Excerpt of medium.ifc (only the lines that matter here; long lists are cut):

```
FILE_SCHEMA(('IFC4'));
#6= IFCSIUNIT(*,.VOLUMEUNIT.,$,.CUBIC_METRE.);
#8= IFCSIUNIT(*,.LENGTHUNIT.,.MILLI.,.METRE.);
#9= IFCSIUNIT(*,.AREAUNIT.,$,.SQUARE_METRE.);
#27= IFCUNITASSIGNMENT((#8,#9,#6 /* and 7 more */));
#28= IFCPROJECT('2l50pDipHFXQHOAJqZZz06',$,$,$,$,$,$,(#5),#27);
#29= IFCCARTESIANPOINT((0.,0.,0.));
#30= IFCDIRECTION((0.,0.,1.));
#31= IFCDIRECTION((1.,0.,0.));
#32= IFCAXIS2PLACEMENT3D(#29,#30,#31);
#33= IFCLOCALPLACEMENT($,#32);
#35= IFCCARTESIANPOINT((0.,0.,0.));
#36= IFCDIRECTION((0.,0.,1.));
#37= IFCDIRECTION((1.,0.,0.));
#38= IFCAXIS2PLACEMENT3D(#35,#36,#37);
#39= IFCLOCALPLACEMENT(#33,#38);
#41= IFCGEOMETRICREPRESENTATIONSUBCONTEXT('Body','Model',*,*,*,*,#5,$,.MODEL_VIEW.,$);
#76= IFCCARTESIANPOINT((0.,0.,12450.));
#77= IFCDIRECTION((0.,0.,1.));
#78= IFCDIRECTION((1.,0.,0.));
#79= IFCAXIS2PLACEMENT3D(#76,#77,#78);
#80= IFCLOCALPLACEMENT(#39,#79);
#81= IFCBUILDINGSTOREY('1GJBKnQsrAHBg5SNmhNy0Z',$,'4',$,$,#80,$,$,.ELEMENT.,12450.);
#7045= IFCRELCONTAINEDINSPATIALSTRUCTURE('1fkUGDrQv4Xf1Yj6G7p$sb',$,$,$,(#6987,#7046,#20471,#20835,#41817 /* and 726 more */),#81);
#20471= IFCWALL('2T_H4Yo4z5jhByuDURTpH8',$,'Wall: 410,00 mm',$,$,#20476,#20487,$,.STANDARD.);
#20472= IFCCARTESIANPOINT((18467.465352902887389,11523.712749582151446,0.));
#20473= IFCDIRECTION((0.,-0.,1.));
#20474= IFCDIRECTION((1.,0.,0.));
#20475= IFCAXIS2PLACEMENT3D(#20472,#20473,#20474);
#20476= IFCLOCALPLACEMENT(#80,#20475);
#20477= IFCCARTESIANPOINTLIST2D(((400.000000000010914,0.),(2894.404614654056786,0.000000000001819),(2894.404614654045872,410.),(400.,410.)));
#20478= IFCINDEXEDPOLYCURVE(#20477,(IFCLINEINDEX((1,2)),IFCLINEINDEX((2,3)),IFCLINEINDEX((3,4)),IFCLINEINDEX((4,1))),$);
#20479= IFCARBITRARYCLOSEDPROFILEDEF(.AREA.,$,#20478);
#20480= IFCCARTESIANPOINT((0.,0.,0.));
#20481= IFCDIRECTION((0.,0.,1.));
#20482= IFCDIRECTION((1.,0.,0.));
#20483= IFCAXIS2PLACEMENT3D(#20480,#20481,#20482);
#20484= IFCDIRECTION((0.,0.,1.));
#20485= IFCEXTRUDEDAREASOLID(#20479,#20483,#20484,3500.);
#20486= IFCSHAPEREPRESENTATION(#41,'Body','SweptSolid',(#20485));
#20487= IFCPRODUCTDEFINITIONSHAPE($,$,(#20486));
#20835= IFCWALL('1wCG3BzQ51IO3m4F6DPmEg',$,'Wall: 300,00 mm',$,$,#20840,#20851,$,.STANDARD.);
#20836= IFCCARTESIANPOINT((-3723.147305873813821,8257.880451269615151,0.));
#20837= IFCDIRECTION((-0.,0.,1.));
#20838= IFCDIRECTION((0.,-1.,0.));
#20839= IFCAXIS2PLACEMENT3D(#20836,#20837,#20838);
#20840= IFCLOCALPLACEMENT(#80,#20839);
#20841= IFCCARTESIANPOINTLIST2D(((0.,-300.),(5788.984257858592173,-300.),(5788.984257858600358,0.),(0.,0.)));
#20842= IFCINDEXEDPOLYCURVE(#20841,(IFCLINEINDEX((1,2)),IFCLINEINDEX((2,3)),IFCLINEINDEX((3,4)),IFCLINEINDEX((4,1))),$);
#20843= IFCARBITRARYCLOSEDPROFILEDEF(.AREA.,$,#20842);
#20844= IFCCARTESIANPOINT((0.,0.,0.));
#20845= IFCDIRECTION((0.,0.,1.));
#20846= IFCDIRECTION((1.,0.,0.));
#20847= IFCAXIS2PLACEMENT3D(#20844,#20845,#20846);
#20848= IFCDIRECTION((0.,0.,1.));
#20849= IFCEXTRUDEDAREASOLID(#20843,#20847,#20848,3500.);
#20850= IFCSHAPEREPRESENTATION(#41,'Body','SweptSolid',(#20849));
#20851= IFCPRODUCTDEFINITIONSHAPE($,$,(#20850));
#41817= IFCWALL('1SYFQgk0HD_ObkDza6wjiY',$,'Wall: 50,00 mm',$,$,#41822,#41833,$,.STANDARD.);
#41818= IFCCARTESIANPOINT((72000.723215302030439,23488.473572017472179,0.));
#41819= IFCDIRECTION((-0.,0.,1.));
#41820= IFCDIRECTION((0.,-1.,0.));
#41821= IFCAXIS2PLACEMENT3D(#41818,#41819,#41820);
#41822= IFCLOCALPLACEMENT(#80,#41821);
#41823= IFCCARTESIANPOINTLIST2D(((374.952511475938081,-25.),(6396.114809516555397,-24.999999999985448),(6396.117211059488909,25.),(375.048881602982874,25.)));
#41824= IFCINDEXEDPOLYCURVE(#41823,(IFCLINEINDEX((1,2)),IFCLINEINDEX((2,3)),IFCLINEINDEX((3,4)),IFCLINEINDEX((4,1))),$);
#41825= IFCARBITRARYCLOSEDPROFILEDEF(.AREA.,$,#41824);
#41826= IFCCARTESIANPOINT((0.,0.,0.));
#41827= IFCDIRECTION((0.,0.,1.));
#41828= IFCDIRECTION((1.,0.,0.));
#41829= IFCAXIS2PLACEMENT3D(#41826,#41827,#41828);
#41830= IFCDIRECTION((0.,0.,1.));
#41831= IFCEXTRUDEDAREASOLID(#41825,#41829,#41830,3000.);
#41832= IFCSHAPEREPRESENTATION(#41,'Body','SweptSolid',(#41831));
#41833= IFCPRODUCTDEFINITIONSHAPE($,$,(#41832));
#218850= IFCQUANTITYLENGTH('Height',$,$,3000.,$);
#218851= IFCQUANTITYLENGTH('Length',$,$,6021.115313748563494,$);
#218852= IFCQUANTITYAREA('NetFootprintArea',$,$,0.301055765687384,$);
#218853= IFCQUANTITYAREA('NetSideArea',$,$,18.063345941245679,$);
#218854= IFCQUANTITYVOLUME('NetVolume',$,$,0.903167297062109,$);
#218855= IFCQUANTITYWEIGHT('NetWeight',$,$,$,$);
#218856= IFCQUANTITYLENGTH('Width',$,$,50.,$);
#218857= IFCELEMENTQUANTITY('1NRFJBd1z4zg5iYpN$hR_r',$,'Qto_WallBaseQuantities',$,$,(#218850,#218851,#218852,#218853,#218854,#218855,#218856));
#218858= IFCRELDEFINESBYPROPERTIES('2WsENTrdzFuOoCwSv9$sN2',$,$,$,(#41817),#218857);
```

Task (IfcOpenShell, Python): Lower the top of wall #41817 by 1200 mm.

```python
import ifcopenshell
import ifcopenshell.api.pset
import ifcopenshell.geom
import ifcopenshell.util.element
import ifcopenshell.util.representation
import ifcopenshell.util.shape
import ifcopenshell.util.unit

model = ifcopenshell.open("medium.ifc")
area_scale = ifcopenshell.util.unit.calculate_unit_scale(model, "AREAUNIT")
volume_scale = ifcopenshell.util.unit.calculate_unit_scale(model, "VOLUMEUNIT")
settings = ifcopenshell.geom.settings()


def volume(element):
    """Net volume in cubic metres, openings subtracted."""
    shape = ifcopenshell.geom.create_shape(settings, element)
    return ifcopenshell.util.shape.get_volume(shape.geometry)


wall = model.by_guid("1SYFQgk0HD_ObkDza6wjiY")
before = volume(wall)

body = ifcopenshell.util.representation.get_representation(wall, "Model", "Body")
solid = body.Items[0]
old_height = solid.Depth
solid.Depth -= 1200.0
after = volume(wall)
thickness = 0.05  # wall thickness in metres

# Update the stored height, areas and volumes.
qto = model.by_id(ifcopenshell.util.element.get_pset(wall, "Qto_WallBaseQuantities", should_inherit=False)["id"])
ifcopenshell.api.pset.edit_qto(model, qto=qto, properties={
    "Height": solid.Depth,
    "NetSideArea": after / thickness / area_scale,
    "NetVolume": after / volume_scale,
})

print(f"height {old_height:g} -> {solid.Depth:g}, volume {before:.3f} -> {after:.3f} m3")

model.write("medium_rev.ifc")
```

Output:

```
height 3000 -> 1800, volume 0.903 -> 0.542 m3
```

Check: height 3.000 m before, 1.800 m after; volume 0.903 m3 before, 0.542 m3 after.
